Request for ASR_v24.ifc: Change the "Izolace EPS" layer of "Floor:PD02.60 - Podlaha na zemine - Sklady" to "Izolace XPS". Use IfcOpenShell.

First a look at what the model holds.

```python
import ifcopenshell
import ifcopenshell.util.element

model = ifcopenshell.open("ASR_v24.ifc")
print(model.schema)
for layer_set in model.by_type("IfcMaterialLayerSet"):
    if layer_set.LayerSetName == "Floor:PD02.60 - Podlaha na zemine - Sklady":
        for layer in layer_set.MaterialLayers:
            print(layer.id(), layer.Material and layer.Material.Name, layer.LayerThickness, sep=" | ")
        print(len(ifcopenshell.util.element.get_elements_by_material(model, layer_set)), "elements and types use it")
print(sorted(m.Name for m in model.by_type("IfcMaterial") if m.Name)[:60])
```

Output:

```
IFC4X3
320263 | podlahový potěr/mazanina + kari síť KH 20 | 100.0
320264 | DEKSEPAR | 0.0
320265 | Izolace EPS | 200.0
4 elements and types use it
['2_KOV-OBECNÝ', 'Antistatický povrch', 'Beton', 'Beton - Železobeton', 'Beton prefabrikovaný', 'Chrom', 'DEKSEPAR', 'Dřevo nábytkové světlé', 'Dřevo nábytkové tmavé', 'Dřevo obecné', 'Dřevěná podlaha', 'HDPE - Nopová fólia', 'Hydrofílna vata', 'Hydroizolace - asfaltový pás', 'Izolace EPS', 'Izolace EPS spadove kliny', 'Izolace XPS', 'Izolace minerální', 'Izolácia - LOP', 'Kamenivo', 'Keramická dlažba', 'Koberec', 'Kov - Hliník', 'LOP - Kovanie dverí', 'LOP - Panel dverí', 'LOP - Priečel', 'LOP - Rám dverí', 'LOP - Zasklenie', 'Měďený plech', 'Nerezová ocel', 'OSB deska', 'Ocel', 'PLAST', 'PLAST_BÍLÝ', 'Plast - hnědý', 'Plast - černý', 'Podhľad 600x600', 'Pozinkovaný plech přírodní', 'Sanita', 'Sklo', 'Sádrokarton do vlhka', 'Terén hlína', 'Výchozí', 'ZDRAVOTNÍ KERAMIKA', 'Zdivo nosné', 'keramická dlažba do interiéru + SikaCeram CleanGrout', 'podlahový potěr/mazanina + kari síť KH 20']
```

```python
import ifcopenshell
import ifcopenshell.api.material

model = ifcopenshell.open("ASR_v24.ifc")

layer_set = next(s for s in model.by_type("IfcMaterialLayerSet") if s.LayerSetName == "Floor:PD02.60 - Podlaha na zemine - Sklady")
layer = next(l for l in layer_set.MaterialLayers if l.Material and l.Material.Name == "Izolace EPS")
material = next(m for m in model.by_type("IfcMaterial") if m.Name == "Izolace XPS")

# Point this one layer at the other material; renaming the old one would change it everywhere.
ifcopenshell.api.material.edit_layer(model, layer=layer, attributes={"Name": material.Name}, material=material)

print([l.Material.Name if l.Material else None for l in layer_set.MaterialLayers])

model.write("ASR_v24_edited.ifc")
```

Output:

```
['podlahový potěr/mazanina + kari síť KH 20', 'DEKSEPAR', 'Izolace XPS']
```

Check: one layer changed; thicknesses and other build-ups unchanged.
